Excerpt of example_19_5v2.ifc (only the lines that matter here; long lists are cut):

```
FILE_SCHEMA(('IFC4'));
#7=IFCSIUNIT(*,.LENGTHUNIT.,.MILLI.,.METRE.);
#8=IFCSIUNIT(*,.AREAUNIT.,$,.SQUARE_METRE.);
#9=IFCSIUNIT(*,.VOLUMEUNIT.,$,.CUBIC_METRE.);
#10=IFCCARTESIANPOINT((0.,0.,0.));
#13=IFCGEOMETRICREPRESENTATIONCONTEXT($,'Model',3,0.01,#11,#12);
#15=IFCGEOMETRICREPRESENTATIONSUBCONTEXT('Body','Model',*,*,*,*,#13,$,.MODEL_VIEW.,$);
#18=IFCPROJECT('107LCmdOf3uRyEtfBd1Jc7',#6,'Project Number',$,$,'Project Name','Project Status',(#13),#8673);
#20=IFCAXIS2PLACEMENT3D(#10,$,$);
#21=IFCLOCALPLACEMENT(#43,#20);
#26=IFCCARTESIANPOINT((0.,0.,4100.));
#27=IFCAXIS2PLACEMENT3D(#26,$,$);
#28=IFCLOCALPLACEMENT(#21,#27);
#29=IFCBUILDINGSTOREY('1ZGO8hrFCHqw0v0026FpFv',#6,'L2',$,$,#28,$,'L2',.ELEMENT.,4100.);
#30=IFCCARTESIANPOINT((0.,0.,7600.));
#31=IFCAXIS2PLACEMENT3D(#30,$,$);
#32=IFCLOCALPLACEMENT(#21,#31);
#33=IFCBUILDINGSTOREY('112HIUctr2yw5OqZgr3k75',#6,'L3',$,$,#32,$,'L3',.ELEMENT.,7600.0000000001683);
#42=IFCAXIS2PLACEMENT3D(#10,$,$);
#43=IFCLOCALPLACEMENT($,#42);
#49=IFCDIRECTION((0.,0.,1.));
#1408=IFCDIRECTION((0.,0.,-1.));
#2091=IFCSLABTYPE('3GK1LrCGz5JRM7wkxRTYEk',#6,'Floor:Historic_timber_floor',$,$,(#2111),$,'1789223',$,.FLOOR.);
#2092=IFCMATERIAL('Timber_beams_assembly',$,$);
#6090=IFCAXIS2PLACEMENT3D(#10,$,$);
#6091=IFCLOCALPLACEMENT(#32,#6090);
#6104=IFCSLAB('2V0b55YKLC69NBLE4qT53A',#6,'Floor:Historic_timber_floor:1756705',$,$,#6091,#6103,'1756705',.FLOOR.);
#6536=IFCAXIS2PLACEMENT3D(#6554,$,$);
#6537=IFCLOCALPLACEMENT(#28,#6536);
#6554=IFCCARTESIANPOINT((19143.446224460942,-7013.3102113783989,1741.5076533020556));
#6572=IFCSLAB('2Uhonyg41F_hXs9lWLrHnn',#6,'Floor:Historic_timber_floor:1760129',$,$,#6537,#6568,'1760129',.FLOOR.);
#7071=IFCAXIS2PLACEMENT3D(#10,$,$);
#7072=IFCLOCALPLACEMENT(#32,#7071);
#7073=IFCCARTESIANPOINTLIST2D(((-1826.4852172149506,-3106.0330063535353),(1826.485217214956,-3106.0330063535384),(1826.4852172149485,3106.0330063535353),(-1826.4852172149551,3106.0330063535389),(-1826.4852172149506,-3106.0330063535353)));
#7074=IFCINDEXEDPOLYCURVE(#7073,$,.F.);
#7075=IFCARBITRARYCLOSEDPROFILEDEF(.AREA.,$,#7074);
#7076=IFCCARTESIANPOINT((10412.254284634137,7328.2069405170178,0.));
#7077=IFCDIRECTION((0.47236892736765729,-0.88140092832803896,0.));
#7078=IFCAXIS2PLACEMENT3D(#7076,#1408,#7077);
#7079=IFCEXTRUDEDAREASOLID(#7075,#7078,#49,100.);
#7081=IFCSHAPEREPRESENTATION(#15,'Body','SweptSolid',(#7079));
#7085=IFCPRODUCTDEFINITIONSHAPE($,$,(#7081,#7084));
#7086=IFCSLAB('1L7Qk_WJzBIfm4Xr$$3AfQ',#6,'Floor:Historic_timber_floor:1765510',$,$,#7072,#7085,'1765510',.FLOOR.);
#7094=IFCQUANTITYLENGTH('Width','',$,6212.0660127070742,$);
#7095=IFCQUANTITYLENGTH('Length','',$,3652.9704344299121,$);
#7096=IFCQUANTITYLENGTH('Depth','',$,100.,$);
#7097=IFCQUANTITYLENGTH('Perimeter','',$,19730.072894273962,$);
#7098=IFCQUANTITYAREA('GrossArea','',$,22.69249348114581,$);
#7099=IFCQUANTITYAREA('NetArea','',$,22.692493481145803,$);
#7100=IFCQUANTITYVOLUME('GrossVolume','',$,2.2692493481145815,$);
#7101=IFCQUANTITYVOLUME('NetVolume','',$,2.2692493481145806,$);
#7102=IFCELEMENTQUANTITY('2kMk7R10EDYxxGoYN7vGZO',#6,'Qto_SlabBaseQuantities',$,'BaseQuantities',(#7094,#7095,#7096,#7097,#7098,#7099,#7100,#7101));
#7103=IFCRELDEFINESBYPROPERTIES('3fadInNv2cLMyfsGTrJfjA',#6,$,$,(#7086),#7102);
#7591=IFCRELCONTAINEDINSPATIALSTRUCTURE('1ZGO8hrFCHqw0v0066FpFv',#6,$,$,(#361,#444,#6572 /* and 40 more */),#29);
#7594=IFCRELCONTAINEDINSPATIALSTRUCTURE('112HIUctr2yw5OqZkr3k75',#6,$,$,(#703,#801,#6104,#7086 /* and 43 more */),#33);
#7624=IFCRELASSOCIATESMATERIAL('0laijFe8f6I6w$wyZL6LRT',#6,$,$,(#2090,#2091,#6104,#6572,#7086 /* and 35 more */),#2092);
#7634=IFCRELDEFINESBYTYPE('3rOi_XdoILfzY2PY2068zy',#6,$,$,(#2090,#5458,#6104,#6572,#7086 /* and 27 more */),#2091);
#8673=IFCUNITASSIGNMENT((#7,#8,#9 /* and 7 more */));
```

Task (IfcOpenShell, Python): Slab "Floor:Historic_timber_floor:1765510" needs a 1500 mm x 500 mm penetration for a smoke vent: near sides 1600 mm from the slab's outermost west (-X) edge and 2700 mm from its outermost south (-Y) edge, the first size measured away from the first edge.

```python
import numpy as np
import ifcopenshell
import ifcopenshell.api.feature
import ifcopenshell.api.geometry
import ifcopenshell.api.pset
import ifcopenshell.api.root
import ifcopenshell.geom
import ifcopenshell.util.element
import ifcopenshell.util.placement
import ifcopenshell.util.representation
import ifcopenshell.util.shape
import ifcopenshell.util.unit

model = ifcopenshell.open("example_19_5v2.ifc")
unit_scale = ifcopenshell.util.unit.calculate_unit_scale(model)
area_scale = ifcopenshell.util.unit.calculate_unit_scale(model, "AREAUNIT")
volume_scale = ifcopenshell.util.unit.calculate_unit_scale(model, "VOLUMEUNIT")
settings = ifcopenshell.geom.settings()


def volume(element):
    """Net volume in cubic metres, openings subtracted."""
    shape = ifcopenshell.geom.create_shape(settings, element)
    return ifcopenshell.util.shape.get_volume(shape.geometry)


slab = model.by_guid("1L7Qk_WJzBIfm4Xr$$3AfQ")
before = volume(slab)

# Extent in the slab's own axes, in metres. The edges named are its -X and -Y sides.
slab_shape = ifcopenshell.geom.create_shape(settings, slab)
vertices = ifcopenshell.util.shape.get_vertices(slab_shape.geometry)
x_min, y_min, bottom = vertices.min(axis=0)
top = vertices[:, 2].max()

opening = ifcopenshell.api.root.create_entity(model, ifc_class="IfcOpeningElement", name="Smoke vent opening", predefined_type="OPENING")
context = ifcopenshell.util.representation.get_context(model, "Model", "Body", "MODEL_VIEW")
width, depth = 1.5, 0.5
outline = [(0.0, 0.0), (width, 0.0), (width, depth), (0.0, depth), (0.0, 0.0)]
# Overshoot both faces by 50 mm so the cut is clean.
shape = ifcopenshell.api.geometry.add_slab_representation(
    model, context=context, depth=top - bottom + 0.1, polyline=outline
)
ifcopenshell.api.geometry.assign_representation(model, product=opening, representation=shape)

matrix = ifcopenshell.util.placement.get_local_placement(slab.ObjectPlacement)
matrix[:, 3] = matrix @ np.append(np.array([x_min + 1.6, y_min + 2.7, bottom - 0.05]) / unit_scale, 1.0)
ifcopenshell.api.geometry.edit_object_placement(model, product=opening, matrix=matrix, is_si=False)
ifcopenshell.api.feature.add_feature(model, feature=opening, element=slab)

after = volume(slab)

# Update the slab's stored quantities.
qto = model.by_id(ifcopenshell.util.element.get_pset(slab, "Qto_SlabBaseQuantities", should_inherit=False)["id"])
ifcopenshell.api.pset.edit_qto(model, qto=qto, properties={
    "NetArea": after / (top - bottom) / area_scale,
    "NetVolume": after / volume_scale,
})

print(f"slab volume {before:.3f} -> {after:.3f} m3")

model.write("example_19_5v2_v2.ifc")
```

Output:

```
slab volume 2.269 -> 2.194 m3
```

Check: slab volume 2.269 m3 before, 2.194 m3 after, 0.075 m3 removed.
